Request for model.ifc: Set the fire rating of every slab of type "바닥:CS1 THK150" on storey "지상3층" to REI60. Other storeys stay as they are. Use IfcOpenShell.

First a look at what the model holds.

```python
import ifcopenshell
import ifcopenshell.util.element

model = ifcopenshell.open("model.ifc")
print(model.schema)
storey = next(s for s in model.by_type("IfcBuildingStorey") if s.Name == "지상3층")
slabs = [e for e in ifcopenshell.util.element.get_decomposition(storey) if e.is_a("IfcSlab")]
seen = {}
for e in slabs:
    element_type = ifcopenshell.util.element.get_type(e)
    key = (element_type.Name if element_type != e and element_type else None, ifcopenshell.util.element.get_pset(e, "Pset_SlabCommon", "FireRating"))
    seen[key] = seen.get(key, 0) + 1
for (name, value), count in sorted(seen.items(), key=str):
    print(count, "x", name, "|", value)
```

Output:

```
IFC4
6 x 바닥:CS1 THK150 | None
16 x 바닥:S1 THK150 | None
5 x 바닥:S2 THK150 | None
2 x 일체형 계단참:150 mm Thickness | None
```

```python
import ifcopenshell
import ifcopenshell.api.pset
import ifcopenshell.util.element

model = ifcopenshell.open("model.ifc")

storey = next(s for s in model.by_type("IfcBuildingStorey") if s.Name == "지상3층")
slabs = [e for e in ifcopenshell.util.element.get_decomposition(storey) if e.is_a("IfcSlab")]

count = 0
for e in slabs:
    element_type = ifcopenshell.util.element.get_type(e)
    if element_type in (None, e) or element_type.Name != "바닥:CS1 THK150":
        continue
    # add_pset returns the element's existing set when there is one.
    pset = ifcopenshell.api.pset.add_pset(model, product=e, name="Pset_SlabCommon")
    ifcopenshell.api.pset.edit_pset(model, pset=pset, properties={"FireRating": "REI60"})
    count += 1

print(count, "slabs updated")

model.write("model_v2.ifc")
```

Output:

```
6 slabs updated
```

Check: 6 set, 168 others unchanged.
